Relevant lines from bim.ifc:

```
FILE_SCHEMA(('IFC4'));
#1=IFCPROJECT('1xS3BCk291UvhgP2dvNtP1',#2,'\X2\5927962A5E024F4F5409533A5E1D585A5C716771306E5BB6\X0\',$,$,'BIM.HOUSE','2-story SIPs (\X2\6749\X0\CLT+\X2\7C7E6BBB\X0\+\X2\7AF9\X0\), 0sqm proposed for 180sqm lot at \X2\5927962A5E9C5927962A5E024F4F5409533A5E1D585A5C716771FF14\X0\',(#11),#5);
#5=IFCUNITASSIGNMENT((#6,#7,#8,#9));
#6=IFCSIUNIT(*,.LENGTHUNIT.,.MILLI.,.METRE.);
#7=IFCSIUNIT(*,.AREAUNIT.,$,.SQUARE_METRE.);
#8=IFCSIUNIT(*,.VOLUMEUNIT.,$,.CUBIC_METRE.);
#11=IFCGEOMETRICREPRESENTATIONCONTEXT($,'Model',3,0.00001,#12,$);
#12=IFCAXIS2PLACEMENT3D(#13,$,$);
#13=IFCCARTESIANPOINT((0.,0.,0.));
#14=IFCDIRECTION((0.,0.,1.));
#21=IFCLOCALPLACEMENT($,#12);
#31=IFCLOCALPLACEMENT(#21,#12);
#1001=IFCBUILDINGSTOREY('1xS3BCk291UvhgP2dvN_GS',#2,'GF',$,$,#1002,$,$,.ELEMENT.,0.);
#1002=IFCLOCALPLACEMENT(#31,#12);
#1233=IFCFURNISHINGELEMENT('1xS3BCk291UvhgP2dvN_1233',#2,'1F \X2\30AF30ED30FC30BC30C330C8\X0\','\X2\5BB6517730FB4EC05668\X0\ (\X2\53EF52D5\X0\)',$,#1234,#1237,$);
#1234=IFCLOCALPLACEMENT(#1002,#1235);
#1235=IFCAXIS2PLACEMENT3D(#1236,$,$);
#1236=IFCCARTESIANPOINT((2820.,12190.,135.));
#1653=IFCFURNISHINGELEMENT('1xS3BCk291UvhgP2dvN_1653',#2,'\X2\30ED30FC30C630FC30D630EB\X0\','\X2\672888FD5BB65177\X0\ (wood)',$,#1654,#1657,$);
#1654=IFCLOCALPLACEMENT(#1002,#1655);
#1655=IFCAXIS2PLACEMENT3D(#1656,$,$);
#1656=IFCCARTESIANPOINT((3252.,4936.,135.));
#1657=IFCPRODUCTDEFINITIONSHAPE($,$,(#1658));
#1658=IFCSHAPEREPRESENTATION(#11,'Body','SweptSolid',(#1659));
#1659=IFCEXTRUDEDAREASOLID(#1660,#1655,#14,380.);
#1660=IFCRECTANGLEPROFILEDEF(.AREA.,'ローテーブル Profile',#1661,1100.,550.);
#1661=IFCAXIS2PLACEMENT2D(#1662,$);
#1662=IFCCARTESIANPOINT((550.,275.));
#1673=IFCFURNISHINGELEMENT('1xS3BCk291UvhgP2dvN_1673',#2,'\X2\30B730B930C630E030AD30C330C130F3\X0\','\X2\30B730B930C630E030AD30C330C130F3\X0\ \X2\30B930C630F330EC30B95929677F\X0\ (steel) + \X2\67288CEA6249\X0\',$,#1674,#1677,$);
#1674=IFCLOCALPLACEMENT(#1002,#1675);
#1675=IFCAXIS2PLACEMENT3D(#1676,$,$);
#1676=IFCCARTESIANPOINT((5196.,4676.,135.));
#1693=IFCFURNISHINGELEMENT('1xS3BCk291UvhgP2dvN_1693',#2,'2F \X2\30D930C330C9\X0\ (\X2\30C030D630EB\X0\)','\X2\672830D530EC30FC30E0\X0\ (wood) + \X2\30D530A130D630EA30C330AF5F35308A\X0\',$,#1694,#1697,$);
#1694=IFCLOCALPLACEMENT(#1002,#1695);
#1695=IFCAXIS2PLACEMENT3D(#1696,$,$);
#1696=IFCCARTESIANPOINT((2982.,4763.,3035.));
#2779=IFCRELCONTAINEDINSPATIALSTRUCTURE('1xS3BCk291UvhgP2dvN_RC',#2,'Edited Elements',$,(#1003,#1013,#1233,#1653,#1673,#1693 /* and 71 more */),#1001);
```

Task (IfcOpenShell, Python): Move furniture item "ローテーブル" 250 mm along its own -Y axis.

```python
import ifcopenshell
import ifcopenshell.api.geometry
import ifcopenshell.util.placement
import ifcopenshell.util.unit

model = ifcopenshell.open("bim.ifc")
unit_scale = ifcopenshell.util.unit.calculate_unit_scale(model)

item = model.by_guid("1xS3BCk291UvhgP2dvN_1653")
matrix = ifcopenshell.util.placement.get_local_placement(item.ObjectPlacement)
matrix[:3, 3] -= matrix[:3, 1] * 0.25 / unit_scale
ifcopenshell.api.geometry.edit_object_placement(model, product=item, matrix=matrix, is_si=False)

print(ifcopenshell.util.placement.get_local_placement(item.ObjectPlacement).round(3) + 0.0)

model.write("bim_v2.ifc")
```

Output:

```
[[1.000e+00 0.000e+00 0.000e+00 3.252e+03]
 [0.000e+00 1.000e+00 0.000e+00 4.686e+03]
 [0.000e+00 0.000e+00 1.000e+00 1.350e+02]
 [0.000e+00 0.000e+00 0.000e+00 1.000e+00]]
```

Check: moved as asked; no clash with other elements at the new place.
